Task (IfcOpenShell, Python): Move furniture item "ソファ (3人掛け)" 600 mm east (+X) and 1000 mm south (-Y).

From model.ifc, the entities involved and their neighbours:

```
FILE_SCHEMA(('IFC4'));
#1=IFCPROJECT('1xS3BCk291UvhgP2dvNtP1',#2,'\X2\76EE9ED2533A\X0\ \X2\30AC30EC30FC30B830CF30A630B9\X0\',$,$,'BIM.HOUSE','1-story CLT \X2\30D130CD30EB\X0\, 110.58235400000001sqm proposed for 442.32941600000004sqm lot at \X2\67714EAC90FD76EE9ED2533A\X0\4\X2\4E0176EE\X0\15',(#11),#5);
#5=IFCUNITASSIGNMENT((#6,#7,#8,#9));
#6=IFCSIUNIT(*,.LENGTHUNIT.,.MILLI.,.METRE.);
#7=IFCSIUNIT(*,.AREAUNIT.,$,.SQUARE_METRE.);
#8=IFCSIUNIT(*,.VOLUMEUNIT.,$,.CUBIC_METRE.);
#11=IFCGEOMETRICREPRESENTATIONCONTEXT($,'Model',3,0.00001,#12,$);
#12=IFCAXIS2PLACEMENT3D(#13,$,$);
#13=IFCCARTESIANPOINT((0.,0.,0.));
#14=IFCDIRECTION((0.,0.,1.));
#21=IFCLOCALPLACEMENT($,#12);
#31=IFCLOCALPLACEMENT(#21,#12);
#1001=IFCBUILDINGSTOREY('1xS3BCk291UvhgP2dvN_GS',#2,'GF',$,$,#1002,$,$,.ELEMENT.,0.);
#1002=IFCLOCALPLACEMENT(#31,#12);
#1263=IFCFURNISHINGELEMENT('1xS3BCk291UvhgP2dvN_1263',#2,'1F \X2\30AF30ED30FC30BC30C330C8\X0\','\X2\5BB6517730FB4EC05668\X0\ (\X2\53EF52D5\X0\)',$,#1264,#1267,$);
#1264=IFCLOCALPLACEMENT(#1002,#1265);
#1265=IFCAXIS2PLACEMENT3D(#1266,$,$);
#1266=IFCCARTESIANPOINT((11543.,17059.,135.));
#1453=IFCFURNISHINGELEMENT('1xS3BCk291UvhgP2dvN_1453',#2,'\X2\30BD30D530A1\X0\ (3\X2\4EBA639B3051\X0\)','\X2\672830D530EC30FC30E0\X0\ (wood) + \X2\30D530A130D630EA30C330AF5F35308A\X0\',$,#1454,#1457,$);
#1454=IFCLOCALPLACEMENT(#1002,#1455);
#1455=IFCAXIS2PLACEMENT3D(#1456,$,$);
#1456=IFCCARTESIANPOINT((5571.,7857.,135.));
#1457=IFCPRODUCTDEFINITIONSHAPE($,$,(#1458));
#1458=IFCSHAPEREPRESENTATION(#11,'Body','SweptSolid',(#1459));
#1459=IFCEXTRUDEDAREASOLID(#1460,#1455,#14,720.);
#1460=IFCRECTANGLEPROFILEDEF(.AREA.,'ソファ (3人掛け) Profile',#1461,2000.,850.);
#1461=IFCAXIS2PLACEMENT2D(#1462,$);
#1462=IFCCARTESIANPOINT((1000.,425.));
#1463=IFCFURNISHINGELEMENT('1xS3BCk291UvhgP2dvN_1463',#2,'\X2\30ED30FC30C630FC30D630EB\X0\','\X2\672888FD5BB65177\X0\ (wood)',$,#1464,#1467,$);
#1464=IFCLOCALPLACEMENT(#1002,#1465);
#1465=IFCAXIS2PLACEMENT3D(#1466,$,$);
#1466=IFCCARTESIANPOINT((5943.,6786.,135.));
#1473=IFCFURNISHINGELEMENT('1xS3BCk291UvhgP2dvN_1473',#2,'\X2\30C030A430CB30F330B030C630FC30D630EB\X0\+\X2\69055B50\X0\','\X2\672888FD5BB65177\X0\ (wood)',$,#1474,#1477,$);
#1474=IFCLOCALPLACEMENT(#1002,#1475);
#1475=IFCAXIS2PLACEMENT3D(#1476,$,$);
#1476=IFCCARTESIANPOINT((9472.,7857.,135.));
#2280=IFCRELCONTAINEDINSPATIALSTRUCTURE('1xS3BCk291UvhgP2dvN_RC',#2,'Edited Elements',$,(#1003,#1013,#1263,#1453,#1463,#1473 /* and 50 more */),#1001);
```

```python
import ifcopenshell
import ifcopenshell.api.geometry
import ifcopenshell.util.placement

model = ifcopenshell.open("model.ifc")

item = model.by_id(1453)
matrix = ifcopenshell.util.placement.get_local_placement(item.ObjectPlacement)
matrix[0, 3] += 600.0
matrix[1, 3] -= 1000.0
ifcopenshell.api.geometry.edit_object_placement(model, product=item, matrix=matrix, is_si=False)

print(ifcopenshell.util.placement.get_local_placement(item.ObjectPlacement).round(3) + 0.0)

model.write("model-out.ifc")
```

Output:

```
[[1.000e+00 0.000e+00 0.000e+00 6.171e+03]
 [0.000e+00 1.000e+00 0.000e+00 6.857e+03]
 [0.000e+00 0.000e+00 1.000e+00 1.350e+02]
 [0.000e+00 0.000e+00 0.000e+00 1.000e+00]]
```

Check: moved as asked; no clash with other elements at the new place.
